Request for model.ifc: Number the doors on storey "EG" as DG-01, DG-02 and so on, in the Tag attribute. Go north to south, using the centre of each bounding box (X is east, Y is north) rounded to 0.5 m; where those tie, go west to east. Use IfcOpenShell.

First a look at what the model holds.

```python
import ifcopenshell
import ifcopenshell.util.element
import ifcopenshell.util.placement

model = ifcopenshell.open("model.ifc")
print(model.schema)
storey = next(s for s in model.by_type("IfcBuildingStorey") if s.Name == "EG")
doors = [e for e in ifcopenshell.util.element.get_decomposition(storey) if e.is_a("IfcDoor")]
for e in sorted(doors, key=lambda e: e.id()):
    origin = ifcopenshell.util.placement.get_local_placement(e.ObjectPlacement)[:3, 3]
    print(e.id(), e.Tag, e.Name, origin.round(2) + 0.0, sep=" | ")
```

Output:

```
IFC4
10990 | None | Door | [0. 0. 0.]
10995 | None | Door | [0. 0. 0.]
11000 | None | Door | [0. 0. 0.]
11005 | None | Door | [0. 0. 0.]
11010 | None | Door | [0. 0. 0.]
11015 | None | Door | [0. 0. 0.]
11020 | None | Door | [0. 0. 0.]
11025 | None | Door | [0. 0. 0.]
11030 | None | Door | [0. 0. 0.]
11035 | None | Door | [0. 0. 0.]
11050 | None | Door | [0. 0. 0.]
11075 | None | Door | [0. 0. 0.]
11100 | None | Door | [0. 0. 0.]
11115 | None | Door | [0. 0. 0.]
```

```python
import ifcopenshell
import ifcopenshell.geom
import ifcopenshell.util.element
import ifcopenshell.util.shape

model = ifcopenshell.open("model.ifc")
settings = ifcopenshell.geom.settings()
settings.set("use-world-coords", True)


def centre(element):
    shape = ifcopenshell.geom.create_shape(settings, element)
    return ifcopenshell.util.shape.get_bbox_centroid(shape.geometry)


storey = next(s for s in model.by_type("IfcBuildingStorey") if s.Name == "EG")
doors = [e for e in ifcopenshell.util.element.get_decomposition(storey) if e.is_a("IfcDoor")]

# Insertion points can sit at a corner or the storey origin, so sort by the geometry (in metres).
centres = {e: centre(e) for e in doors}
doors.sort(key=lambda e: (-round(centres[e][1] / 0.5), centres[e][0]))

for i, e in enumerate(doors, start=1):
    number = f"DG-{i:02d}"
    e.Tag = number
    print(e.id(), number)

model.write("model_v2.ifc")
```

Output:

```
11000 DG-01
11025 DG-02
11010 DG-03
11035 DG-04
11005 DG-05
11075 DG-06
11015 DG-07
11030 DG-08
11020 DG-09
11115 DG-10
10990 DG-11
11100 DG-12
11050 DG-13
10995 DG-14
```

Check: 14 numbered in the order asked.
